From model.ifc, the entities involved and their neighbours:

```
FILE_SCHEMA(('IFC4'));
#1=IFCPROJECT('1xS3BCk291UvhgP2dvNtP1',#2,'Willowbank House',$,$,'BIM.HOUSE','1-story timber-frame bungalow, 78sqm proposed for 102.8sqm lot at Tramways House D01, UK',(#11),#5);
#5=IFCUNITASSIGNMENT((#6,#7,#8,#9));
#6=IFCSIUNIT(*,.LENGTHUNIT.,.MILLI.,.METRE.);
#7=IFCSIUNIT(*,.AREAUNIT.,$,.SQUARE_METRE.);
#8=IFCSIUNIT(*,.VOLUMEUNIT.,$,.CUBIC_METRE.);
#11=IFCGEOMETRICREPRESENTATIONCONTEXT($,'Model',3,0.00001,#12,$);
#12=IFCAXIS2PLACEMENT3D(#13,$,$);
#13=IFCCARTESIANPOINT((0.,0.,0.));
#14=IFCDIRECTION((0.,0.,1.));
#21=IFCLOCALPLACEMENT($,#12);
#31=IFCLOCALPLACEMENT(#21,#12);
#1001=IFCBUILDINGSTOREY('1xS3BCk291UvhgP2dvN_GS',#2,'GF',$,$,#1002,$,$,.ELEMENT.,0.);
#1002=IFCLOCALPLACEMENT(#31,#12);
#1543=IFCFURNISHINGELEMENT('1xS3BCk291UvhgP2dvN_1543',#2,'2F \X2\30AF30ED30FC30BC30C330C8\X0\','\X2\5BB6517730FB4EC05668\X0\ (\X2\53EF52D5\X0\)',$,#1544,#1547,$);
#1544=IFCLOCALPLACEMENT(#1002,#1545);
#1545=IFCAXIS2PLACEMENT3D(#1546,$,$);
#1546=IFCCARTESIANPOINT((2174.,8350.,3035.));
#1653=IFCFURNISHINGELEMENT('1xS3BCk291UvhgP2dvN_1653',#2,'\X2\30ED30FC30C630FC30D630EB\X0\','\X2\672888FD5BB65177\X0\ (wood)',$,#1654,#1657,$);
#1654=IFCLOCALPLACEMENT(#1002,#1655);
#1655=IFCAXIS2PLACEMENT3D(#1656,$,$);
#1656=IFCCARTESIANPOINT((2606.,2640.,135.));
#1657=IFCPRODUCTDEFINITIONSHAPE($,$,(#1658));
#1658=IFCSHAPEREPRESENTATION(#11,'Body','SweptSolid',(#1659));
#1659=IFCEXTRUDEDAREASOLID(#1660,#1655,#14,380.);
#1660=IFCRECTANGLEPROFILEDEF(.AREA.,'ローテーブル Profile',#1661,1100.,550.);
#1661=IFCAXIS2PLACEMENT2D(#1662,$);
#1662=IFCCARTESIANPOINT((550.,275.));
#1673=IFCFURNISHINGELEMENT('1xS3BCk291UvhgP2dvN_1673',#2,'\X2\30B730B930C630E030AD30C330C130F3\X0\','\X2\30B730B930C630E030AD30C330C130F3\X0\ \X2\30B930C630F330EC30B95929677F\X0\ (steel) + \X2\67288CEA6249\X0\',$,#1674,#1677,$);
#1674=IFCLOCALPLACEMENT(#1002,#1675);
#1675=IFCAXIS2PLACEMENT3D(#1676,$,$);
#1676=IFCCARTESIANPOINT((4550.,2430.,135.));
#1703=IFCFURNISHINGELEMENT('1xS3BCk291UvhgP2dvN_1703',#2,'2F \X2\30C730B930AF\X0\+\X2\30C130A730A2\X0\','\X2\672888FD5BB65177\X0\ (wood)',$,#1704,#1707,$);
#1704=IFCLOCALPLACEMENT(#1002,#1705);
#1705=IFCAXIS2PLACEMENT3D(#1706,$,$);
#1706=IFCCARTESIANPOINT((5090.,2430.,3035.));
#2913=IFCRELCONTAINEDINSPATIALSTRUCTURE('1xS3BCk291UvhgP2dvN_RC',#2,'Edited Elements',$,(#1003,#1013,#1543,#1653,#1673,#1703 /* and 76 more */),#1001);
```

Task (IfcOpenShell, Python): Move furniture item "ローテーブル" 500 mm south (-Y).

```python
import ifcopenshell
import ifcopenshell.api.geometry
import ifcopenshell.util.placement
import ifcopenshell.util.unit

model = ifcopenshell.open("model.ifc")
unit_scale = ifcopenshell.util.unit.calculate_unit_scale(model)

item = model.by_guid("1xS3BCk291UvhgP2dvN_1653")
matrix = ifcopenshell.util.placement.get_local_placement(item.ObjectPlacement)
matrix[1, 3] -= 0.5 / unit_scale
ifcopenshell.api.geometry.edit_object_placement(model, product=item, matrix=matrix, is_si=False)

print(ifcopenshell.util.placement.get_local_placement(item.ObjectPlacement).round(3) + 0.0)

model.write("model_rev.ifc")
```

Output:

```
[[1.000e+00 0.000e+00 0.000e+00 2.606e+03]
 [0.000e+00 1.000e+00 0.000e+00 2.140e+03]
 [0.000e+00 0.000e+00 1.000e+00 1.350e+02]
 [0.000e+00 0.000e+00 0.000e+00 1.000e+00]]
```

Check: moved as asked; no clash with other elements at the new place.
